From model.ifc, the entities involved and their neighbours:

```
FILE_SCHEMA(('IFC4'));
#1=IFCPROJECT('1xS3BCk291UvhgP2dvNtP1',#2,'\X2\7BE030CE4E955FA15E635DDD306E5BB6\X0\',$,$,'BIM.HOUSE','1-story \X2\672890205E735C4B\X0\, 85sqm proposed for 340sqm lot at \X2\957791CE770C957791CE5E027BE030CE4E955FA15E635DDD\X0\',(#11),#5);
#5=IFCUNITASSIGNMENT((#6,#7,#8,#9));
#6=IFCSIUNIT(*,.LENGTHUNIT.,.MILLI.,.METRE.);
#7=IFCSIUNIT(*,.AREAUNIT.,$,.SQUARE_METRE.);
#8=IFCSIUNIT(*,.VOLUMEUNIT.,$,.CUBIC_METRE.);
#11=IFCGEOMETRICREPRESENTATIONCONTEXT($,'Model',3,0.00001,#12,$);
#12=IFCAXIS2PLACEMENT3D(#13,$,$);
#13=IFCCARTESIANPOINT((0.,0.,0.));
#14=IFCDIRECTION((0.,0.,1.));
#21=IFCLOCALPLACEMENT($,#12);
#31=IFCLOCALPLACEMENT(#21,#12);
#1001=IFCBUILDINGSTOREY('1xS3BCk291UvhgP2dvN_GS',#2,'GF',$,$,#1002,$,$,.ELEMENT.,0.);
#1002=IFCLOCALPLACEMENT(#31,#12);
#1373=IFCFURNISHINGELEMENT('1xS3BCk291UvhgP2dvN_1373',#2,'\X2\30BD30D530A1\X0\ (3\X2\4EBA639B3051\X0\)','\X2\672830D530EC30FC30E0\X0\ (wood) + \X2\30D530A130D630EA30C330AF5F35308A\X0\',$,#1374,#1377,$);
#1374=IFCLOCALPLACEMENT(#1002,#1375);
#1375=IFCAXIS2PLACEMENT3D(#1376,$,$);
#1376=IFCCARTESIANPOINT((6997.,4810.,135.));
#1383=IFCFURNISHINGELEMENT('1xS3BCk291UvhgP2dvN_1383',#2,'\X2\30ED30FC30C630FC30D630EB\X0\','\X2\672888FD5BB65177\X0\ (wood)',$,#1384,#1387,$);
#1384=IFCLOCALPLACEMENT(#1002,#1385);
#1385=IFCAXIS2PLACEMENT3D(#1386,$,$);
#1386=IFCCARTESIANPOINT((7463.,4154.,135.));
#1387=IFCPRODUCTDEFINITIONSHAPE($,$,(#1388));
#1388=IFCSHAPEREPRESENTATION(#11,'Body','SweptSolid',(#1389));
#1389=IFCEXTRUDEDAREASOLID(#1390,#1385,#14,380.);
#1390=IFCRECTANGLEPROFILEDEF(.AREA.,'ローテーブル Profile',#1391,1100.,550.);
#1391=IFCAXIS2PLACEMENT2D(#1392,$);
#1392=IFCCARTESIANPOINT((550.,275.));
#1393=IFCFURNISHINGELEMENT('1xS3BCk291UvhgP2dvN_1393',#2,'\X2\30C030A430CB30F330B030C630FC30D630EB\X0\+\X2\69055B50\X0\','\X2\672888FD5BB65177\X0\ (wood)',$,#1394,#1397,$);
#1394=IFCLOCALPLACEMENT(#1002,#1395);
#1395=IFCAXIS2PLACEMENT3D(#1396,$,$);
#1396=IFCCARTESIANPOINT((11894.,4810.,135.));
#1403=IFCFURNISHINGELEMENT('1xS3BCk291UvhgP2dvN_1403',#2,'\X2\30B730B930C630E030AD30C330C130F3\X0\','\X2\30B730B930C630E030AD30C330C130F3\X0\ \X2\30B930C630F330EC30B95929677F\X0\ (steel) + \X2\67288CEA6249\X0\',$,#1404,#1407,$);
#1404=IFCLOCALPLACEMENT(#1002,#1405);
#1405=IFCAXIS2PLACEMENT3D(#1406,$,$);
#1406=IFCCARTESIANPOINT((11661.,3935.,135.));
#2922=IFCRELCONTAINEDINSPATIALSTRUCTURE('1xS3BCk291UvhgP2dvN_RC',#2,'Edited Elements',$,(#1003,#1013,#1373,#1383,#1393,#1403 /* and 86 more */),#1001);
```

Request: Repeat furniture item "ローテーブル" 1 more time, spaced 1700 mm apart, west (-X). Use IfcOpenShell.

```python
import numpy as np
import ifcopenshell
import ifcopenshell.api.geometry
import ifcopenshell.api.root
import ifcopenshell.util.element
import ifcopenshell.util.placement
import ifcopenshell.util.unit

model = ifcopenshell.open("model.ifc")
unit_scale = ifcopenshell.util.unit.calculate_unit_scale(model)


def reuse_history(source, copy):
    """copy_class also copies each property set's owner history, people and application; keep the originals."""
    for rel in copy.IsDefinedBy:
        if rel.is_a("IfcRelDefinesByProperties") and (history := rel.RelatingPropertyDefinition.OwnerHistory):
            rel.RelatingPropertyDefinition.OwnerHistory = source.OwnerHistory
            ifcopenshell.util.element.remove_deep2(model, history)


source = model.by_guid("1xS3BCk291UvhgP2dvN_1383")
base = ifcopenshell.util.placement.get_local_placement(source.ObjectPlacement)
step = np.array([-1.0, 0.0, 0.0]) * 1.7 / unit_scale

for i in range(1, 2):
    copy = ifcopenshell.api.root.copy_class(model, product=source)
    copy.Representation = ifcopenshell.util.element.copy_deep(
        model, source.Representation, exclude=["IfcGeometricRepresentationContext", "IfcRepresentationMap"]
    )
    reuse_history(source, copy)
    matrix = base.copy()
    matrix[:3, 3] += i * step
    print("added at", matrix[:3, 3].round(3) + 0.0)
    ifcopenshell.api.geometry.edit_object_placement(model, product=copy, matrix=matrix, is_si=False)

model.write("model_edited.ifc")
```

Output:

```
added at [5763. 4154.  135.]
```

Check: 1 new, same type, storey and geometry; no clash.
